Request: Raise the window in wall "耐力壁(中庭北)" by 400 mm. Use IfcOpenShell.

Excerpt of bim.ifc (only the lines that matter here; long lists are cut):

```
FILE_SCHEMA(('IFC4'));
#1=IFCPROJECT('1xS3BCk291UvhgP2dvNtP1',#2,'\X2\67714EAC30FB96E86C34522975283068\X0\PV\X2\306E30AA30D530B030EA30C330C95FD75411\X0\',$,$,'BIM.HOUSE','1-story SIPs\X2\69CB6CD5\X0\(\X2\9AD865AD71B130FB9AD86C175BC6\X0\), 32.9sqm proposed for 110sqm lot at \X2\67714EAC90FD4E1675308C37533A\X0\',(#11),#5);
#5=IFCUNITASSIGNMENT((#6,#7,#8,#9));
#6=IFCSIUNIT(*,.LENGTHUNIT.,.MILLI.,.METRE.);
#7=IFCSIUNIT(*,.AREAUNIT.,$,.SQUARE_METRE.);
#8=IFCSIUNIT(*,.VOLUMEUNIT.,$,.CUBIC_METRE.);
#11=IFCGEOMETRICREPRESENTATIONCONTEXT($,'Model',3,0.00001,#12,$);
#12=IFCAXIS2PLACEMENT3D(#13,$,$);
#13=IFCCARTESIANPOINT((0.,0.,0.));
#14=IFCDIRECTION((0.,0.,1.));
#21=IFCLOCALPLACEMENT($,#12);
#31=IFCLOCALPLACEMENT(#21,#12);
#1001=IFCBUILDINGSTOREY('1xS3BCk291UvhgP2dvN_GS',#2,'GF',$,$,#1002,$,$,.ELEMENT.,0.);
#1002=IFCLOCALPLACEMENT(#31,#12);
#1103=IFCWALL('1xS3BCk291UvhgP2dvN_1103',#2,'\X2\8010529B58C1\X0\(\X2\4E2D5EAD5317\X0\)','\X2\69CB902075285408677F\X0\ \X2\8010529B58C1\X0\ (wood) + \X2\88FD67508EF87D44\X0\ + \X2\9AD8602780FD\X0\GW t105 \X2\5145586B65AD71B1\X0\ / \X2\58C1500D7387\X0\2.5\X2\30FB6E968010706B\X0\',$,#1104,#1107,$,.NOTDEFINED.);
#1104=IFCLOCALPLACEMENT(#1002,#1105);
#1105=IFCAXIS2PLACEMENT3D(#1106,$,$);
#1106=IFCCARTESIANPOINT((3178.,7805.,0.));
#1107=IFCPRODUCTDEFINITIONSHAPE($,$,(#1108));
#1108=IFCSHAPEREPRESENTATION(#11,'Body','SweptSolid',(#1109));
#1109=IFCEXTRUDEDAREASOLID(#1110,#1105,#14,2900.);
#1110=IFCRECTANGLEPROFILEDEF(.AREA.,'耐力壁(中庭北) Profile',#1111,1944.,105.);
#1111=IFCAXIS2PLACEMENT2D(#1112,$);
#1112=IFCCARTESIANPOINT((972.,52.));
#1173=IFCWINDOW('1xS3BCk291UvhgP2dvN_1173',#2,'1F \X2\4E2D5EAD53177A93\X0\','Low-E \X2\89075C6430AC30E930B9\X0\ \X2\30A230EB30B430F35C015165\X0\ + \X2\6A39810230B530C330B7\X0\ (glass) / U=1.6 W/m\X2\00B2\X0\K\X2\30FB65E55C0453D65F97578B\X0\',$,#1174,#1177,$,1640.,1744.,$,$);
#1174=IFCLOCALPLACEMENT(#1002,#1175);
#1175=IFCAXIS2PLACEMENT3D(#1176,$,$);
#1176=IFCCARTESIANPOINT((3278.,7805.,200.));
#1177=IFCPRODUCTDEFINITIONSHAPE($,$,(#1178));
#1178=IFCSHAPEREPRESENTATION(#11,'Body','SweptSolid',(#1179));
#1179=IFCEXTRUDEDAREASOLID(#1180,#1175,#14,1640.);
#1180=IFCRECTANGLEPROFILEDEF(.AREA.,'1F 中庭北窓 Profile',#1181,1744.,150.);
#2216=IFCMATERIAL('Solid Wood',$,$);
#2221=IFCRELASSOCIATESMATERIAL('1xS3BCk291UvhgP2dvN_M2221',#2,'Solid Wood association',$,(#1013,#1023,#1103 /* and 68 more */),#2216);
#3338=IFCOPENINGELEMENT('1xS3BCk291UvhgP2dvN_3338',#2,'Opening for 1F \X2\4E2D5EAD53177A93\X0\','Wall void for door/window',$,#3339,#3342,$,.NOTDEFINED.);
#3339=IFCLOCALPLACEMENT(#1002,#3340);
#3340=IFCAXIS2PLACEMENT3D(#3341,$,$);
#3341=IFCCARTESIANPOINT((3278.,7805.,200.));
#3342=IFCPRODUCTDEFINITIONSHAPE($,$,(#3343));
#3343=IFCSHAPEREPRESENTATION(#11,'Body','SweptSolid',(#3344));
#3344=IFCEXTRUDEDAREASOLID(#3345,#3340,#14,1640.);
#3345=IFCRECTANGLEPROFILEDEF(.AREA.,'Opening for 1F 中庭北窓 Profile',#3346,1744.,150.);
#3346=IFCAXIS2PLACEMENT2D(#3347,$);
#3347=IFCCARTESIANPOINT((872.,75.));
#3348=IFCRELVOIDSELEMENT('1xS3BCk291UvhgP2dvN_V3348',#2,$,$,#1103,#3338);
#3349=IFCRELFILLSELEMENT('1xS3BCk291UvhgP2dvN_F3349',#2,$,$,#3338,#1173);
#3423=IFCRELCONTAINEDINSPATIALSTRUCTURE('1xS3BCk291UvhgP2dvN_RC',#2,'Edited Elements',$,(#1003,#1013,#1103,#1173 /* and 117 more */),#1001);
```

```python
import numpy as np
import ifcopenshell
import ifcopenshell.api.geometry
import ifcopenshell.util.placement
import ifcopenshell.util.unit

model = ifcopenshell.open("bim.ifc")
unit_scale = ifcopenshell.util.unit.calculate_unit_scale(model)

window = model.by_id(1173)
opening = window.FillsVoids[0].RelatingOpeningElement
dz = 0.4 / unit_scale

shift = np.array([0.0, 0.0, dz])
# The window is not placed relative to its opening, so move both.
for product in (opening, window):
    matrix = ifcopenshell.util.placement.get_local_placement(product.ObjectPlacement)
    matrix[:3, 3] += shift
    ifcopenshell.api.geometry.edit_object_placement(model, product=product, matrix=matrix, is_si=False)

print(f"moved by {dz * unit_scale:+.3f} m")

model.write("bim_updated.ifc")
```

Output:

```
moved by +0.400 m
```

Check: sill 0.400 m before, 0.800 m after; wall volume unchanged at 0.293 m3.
